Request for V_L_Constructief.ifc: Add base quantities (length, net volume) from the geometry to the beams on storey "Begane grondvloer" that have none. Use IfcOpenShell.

First a look at what the model holds.

```python
import ifcopenshell
import ifcopenshell.util.element
import ifcopenshell.util.unit

model = ifcopenshell.open("V_L_Constructief.ifc")
print(model.schema)
for unit_type in ("LENGTHUNIT", "AREAUNIT", "VOLUMEUNIT"):
    print(unit_type, ifcopenshell.util.unit.calculate_unit_scale(model, unit_type))
storey = next(s for s in model.by_type("IfcBuildingStorey") if s.Name == "Begane grondvloer")
beams = [e for e in ifcopenshell.util.element.get_decomposition(storey) if e.is_a("IfcBeam")]
for e in sorted(beams, key=lambda e: e.id()):
    print(e.id(), e.is_a(), e.Name, list(ifcopenshell.util.element.get_psets(e, qtos_only=True)), sep=" | ")
```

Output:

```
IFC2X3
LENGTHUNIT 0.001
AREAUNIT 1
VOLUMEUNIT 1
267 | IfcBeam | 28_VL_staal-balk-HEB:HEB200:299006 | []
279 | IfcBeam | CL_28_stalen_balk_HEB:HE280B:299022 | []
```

```python
import ifcopenshell
import ifcopenshell.api.pset
import ifcopenshell.geom
import ifcopenshell.util.element
import ifcopenshell.util.shape
import ifcopenshell.util.unit

model = ifcopenshell.open("V_L_Constructief.ifc")
unit_scale = ifcopenshell.util.unit.calculate_unit_scale(model)
volume_scale = ifcopenshell.util.unit.calculate_unit_scale(model, "VOLUMEUNIT")
settings = ifcopenshell.geom.settings()

storey = next(s for s in model.by_type("IfcBuildingStorey") if s.Name == "Begane grondvloer")
beams = [e for e in ifcopenshell.util.element.get_decomposition(storey) if e.is_a("IfcBeam")]

for e in sorted(beams, key=lambda e: e.id()):
    if ifcopenshell.util.element.get_psets(e, qtos_only=True, should_inherit=False):
        continue
    # Geometry comes back in metres, in the element's own axes.
    shape = ifcopenshell.geom.create_shape(settings, e)
    values = {
        "Length": ifcopenshell.util.shape.get_max_xyz(shape.geometry) / unit_scale,
        "NetVolume": ifcopenshell.util.shape.get_volume(shape.geometry) / volume_scale,
    }
    qto = ifcopenshell.api.pset.add_qto(model, product=e, name="BaseQuantities")
    ifcopenshell.api.pset.edit_qto(model, qto=qto, properties=values)
    print(e.id(), {k: round(v, 3) for k, v in values.items()})

model.write("V_L_Constructief_updated.ifc")
```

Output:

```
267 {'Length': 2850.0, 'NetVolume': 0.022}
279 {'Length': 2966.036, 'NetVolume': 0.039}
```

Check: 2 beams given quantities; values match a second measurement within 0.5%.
